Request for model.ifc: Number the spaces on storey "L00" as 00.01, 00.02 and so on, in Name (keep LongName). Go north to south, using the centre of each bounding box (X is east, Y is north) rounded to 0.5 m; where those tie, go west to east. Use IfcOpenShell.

First a look at what the model holds.

```python
import ifcopenshell
import ifcopenshell.util.element
import ifcopenshell.util.placement

model = ifcopenshell.open("model.ifc")
print(model.schema)
storey = next(s for s in model.by_type("IfcBuildingStorey") if s.Name == "L00")
spaces = [e for e in ifcopenshell.util.element.get_decomposition(storey) if e.is_a("IfcSpace")]
for e in sorted(spaces, key=lambda e: e.id()):
    origin = ifcopenshell.util.placement.get_local_placement(e.ObjectPlacement)[:3, 3]
    print(e.id(), e.Name, e.LongName, origin.round(2) + 0.0, sep=" | ")
```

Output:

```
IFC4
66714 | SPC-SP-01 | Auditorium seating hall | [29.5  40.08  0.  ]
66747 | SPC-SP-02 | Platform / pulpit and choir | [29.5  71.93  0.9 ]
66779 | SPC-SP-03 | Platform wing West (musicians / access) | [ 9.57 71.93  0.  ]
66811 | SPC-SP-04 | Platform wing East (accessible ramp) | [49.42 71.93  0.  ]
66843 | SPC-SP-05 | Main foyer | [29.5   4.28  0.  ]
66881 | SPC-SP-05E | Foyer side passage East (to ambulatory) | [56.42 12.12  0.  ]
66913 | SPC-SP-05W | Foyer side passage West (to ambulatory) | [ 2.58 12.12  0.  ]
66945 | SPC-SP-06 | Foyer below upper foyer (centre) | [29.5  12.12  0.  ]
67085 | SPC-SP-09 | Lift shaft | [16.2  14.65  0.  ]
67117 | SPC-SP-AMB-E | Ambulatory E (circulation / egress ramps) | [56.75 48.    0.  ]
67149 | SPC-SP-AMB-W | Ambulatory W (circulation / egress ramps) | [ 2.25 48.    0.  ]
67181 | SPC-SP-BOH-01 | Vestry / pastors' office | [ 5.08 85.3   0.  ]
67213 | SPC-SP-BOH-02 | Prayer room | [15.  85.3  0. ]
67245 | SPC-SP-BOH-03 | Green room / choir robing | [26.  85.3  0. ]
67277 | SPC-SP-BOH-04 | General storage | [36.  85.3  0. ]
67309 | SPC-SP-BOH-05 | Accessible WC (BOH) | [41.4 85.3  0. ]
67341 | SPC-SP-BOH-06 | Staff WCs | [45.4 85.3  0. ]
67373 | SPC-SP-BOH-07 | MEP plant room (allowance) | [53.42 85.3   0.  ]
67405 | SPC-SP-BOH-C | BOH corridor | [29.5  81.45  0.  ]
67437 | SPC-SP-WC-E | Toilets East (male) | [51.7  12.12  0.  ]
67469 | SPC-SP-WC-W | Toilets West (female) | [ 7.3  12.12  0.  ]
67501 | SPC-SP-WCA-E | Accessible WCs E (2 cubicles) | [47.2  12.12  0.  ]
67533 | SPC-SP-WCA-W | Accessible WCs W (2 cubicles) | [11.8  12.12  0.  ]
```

```python
import ifcopenshell
import ifcopenshell.geom
import ifcopenshell.util.element
import ifcopenshell.util.shape

model = ifcopenshell.open("model.ifc")
settings = ifcopenshell.geom.settings()
settings.set("use-world-coords", True)


def centre(element):
    shape = ifcopenshell.geom.create_shape(settings, element)
    return ifcopenshell.util.shape.get_bbox_centroid(shape.geometry)


storey = next(s for s in model.by_type("IfcBuildingStorey") if s.Name == "L00")
spaces = [e for e in ifcopenshell.util.element.get_decomposition(storey) if e.is_a("IfcSpace")]

# Insertion points can sit at a corner or the storey origin, so sort by the geometry (in metres).
centres = {e: centre(e) for e in spaces}
spaces.sort(key=lambda e: (-round(centres[e][1] / 0.5), centres[e][0]))

for i, e in enumerate(spaces, start=1):
    number = f"00.{i:02d}"
    e.Name = number
    print(e.id(), number)

model.write("model_edited.ifc")
```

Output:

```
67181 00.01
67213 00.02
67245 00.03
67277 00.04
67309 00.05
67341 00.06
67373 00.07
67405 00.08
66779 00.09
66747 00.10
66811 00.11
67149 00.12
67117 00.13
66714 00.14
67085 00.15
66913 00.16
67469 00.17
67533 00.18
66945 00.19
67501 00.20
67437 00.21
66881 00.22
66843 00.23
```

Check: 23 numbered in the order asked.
